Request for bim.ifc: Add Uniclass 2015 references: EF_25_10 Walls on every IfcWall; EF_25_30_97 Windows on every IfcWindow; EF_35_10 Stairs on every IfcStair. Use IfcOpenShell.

First a look at what the model holds.

```python
import ifcopenshell

model = ifcopenshell.open("bim.ifc")
print(model.schema)
print("classifications:", [c.Name for c in model.by_type("IfcClassification")])
for ifc_class in ("IfcDoor", "IfcRoof", "IfcStair", "IfcWall", "IfcWindow"):
    print(ifc_class, len(model.by_type(ifc_class)))
```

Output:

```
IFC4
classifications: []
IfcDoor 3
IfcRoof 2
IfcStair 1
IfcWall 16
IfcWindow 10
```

```python
import ifcopenshell
import ifcopenshell.api.classification

model = ifcopenshell.open("bim.ifc")

system = ifcopenshell.api.classification.add_classification(model, classification="Uniclass 2015")

codes = {
    "IfcWall": ("EF_25_10", "Walls"),
    "IfcWindow": ("EF_25_30_97", "Windows"),
    "IfcStair": ("EF_35_10", "Stairs"),
}
for ifc_class, (code, name) in codes.items():
    products = model.by_type(ifc_class)
    ifcopenshell.api.classification.add_reference(
        model, products=products, classification=system, identification=code, name=name
    )
    print(code, len(products))

model.write("bim_v2.ifc")
```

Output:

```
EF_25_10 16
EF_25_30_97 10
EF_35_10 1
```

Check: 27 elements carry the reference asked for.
